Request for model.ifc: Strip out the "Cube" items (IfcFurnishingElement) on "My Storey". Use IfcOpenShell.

First a look at what the model holds.

```python
import ifcopenshell
import ifcopenshell.util.element

model = ifcopenshell.open("model.ifc")
print(model.schema)
storey = next(s for s in model.by_type("IfcBuildingStorey") if s.Name == "My Storey")
furniture = [e for e in ifcopenshell.util.element.get_decomposition(storey) if e.is_a("IfcFurnishingElement")]
seen = {}
for e in furniture:
    element_type = ifcopenshell.util.element.get_type(e)
    name = element_type.Name if element_type not in (None, e) else None
    seen[name] = seen.get(name, 0) + 1
for name, count in sorted(seen.items(), key=str):
    print(count, "x", name)
```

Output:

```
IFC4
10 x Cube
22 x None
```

```python
import ifcopenshell
import ifcopenshell.api.root
import ifcopenshell.util.element

model = ifcopenshell.open("model.ifc")

storey = next(s for s in model.by_type("IfcBuildingStorey") if s.Name == "My Storey")
furniture = [e for e in ifcopenshell.util.element.get_decomposition(storey) if e.is_a("IfcFurnishingElement")]
targets = [e for e in furniture if (t := ifcopenshell.util.element.get_type(e)) not in (None, e) and t.Name == "Cube"]

for e in targets:
    ifcopenshell.api.root.remove_product(model, product=e)
print(len(targets), "removed")

model.write("model_edited.ifc")
```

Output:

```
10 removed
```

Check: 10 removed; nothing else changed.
